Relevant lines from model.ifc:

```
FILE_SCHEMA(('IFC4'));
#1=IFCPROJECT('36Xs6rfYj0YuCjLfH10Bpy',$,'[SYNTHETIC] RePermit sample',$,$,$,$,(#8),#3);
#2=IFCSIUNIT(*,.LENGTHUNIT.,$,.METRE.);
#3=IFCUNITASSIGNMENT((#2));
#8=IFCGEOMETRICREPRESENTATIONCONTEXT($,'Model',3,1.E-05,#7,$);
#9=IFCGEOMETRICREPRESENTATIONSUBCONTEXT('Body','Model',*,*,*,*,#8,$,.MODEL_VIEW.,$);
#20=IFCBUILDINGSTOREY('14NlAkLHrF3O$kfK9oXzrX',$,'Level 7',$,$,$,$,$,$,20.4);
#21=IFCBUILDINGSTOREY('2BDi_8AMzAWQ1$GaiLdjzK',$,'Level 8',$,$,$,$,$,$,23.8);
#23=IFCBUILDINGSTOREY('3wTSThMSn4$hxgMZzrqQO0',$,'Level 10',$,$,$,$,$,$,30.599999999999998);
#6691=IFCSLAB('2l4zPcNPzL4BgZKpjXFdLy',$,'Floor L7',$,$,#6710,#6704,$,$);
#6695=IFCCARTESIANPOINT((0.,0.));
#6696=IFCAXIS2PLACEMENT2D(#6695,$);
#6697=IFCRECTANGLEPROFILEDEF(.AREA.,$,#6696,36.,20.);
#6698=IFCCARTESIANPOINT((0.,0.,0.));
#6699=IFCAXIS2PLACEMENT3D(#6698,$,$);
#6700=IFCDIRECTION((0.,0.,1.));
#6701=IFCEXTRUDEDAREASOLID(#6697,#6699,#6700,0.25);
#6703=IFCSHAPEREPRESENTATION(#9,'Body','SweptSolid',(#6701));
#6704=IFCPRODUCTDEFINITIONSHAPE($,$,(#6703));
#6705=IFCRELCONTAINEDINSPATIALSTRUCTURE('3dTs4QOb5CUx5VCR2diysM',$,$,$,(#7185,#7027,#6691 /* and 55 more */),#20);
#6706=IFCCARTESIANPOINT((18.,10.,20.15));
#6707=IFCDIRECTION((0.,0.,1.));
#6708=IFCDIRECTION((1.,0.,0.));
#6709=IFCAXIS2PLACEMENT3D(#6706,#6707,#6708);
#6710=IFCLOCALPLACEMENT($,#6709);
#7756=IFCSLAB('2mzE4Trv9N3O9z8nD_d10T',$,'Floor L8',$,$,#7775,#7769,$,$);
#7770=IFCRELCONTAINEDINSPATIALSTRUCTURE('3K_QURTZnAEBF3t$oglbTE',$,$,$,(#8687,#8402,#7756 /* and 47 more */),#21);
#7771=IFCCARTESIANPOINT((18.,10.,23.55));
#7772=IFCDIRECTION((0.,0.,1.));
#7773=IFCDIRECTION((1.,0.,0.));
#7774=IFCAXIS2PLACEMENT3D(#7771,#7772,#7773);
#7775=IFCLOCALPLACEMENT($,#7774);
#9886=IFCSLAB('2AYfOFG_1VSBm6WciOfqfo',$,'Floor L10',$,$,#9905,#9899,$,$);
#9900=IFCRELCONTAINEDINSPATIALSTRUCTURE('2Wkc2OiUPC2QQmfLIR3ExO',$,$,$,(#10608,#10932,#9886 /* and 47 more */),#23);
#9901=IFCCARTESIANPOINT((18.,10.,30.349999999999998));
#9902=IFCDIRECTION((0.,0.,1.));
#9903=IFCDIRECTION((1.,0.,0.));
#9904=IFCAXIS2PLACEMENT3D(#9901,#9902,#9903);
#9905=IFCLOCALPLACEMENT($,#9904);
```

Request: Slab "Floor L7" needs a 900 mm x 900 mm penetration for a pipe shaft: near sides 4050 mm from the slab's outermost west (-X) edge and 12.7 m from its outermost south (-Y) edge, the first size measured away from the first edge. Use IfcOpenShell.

```python
import numpy as np
import ifcopenshell
import ifcopenshell.api.feature
import ifcopenshell.api.geometry
import ifcopenshell.api.root
import ifcopenshell.geom
import ifcopenshell.util.placement
import ifcopenshell.util.representation
import ifcopenshell.util.shape
import ifcopenshell.util.unit

model = ifcopenshell.open("model.ifc")
unit_scale = ifcopenshell.util.unit.calculate_unit_scale(model)
settings = ifcopenshell.geom.settings()


def volume(element):
    """Net volume in cubic metres, openings subtracted."""
    shape = ifcopenshell.geom.create_shape(settings, element)
    return ifcopenshell.util.shape.get_volume(shape.geometry)


slab = model.by_guid("2l4zPcNPzL4BgZKpjXFdLy")
before = volume(slab)

# Extent in the slab's own axes, in metres. The edges named are its -X and -Y sides.
slab_shape = ifcopenshell.geom.create_shape(settings, slab)
vertices = ifcopenshell.util.shape.get_vertices(slab_shape.geometry)
x_min, y_min, bottom = vertices.min(axis=0)
top = vertices[:, 2].max()

opening = ifcopenshell.api.root.create_entity(model, ifc_class="IfcOpeningElement", name="Pipe shaft opening", predefined_type="OPENING")
context = ifcopenshell.util.representation.get_context(model, "Model", "Body", "MODEL_VIEW")
width, depth = 0.9, 0.9
outline = [(0.0, 0.0), (width, 0.0), (width, depth), (0.0, depth), (0.0, 0.0)]
# Overshoot both faces by 50 mm so the cut is clean.
shape = ifcopenshell.api.geometry.add_slab_representation(
    model, context=context, depth=top - bottom + 0.1, polyline=outline
)
ifcopenshell.api.geometry.assign_representation(model, product=opening, representation=shape)

matrix = ifcopenshell.util.placement.get_local_placement(slab.ObjectPlacement)
matrix[:, 3] = matrix @ np.append(np.array([x_min + 4.05, y_min + 12.7, bottom - 0.05]) / unit_scale, 1.0)
ifcopenshell.api.geometry.edit_object_placement(model, product=opening, matrix=matrix, is_si=False)
ifcopenshell.api.feature.add_feature(model, feature=opening, element=slab)

after = volume(slab)

print(f"slab volume {before:.3f} -> {after:.3f} m3")

model.write("model_updated.ifc")
```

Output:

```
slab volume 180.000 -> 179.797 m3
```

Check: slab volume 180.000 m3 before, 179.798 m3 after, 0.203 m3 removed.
